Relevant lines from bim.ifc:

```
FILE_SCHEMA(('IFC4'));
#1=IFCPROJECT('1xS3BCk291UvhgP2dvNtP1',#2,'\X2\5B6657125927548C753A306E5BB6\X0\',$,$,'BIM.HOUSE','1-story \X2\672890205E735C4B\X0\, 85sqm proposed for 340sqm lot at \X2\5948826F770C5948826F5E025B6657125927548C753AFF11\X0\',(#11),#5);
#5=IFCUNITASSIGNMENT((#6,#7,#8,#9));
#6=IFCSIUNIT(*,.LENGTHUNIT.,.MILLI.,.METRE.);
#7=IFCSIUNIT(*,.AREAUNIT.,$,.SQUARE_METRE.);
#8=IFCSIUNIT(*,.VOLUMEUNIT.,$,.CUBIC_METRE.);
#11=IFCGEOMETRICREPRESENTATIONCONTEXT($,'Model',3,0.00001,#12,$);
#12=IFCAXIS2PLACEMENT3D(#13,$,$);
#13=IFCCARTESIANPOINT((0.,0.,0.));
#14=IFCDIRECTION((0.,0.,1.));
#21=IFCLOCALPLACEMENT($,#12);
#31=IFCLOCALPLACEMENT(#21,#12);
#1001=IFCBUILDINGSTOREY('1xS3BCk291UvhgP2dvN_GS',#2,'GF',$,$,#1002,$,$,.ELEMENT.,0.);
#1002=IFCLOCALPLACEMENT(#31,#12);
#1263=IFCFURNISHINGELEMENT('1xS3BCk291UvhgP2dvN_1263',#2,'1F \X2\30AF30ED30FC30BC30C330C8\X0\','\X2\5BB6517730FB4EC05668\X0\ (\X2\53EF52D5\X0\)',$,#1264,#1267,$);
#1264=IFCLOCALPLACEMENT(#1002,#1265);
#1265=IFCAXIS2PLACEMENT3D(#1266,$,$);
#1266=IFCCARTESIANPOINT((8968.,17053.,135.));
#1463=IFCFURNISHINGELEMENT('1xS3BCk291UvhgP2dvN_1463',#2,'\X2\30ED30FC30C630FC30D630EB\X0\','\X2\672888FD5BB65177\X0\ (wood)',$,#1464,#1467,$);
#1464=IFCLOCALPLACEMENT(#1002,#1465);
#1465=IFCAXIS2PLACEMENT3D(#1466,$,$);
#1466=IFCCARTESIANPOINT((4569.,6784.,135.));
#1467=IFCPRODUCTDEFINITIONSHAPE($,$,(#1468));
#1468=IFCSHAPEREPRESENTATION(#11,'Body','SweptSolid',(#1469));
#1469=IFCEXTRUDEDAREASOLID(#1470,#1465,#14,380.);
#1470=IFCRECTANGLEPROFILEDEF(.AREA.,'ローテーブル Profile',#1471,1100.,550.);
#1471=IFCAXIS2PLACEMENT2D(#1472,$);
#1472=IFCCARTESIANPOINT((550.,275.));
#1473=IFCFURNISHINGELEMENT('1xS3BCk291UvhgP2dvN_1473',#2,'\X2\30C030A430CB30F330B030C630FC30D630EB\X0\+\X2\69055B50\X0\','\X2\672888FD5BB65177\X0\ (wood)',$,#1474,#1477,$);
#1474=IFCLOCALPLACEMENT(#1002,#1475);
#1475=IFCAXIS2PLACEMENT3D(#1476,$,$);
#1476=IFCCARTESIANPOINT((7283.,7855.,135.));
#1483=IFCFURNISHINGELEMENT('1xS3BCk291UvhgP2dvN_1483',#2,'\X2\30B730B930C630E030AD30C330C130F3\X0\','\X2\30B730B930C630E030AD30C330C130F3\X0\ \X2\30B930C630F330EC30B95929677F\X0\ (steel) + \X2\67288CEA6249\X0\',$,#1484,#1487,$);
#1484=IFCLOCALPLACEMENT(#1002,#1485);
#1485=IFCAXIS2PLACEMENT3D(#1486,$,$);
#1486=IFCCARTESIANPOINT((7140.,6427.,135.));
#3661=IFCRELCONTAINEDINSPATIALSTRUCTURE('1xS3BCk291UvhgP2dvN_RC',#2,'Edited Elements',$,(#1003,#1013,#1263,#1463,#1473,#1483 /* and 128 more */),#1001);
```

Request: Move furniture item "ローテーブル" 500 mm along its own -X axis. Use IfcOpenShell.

```python
import ifcopenshell
import ifcopenshell.api.geometry
import ifcopenshell.util.placement

model = ifcopenshell.open("bim.ifc")

item = model.by_guid("1xS3BCk291UvhgP2dvN_1463")
matrix = ifcopenshell.util.placement.get_local_placement(item.ObjectPlacement)
matrix[:3, 3] -= matrix[:3, 0] * 500.0
ifcopenshell.api.geometry.edit_object_placement(model, product=item, matrix=matrix, is_si=False)

print(ifcopenshell.util.placement.get_local_placement(item.ObjectPlacement).round(3) + 0.0)

model.write("bim_rev.ifc")
```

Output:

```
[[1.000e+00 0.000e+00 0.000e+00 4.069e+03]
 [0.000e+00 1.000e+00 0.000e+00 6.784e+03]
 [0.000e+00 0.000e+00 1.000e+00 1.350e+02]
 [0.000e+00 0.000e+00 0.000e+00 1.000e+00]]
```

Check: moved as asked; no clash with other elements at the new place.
